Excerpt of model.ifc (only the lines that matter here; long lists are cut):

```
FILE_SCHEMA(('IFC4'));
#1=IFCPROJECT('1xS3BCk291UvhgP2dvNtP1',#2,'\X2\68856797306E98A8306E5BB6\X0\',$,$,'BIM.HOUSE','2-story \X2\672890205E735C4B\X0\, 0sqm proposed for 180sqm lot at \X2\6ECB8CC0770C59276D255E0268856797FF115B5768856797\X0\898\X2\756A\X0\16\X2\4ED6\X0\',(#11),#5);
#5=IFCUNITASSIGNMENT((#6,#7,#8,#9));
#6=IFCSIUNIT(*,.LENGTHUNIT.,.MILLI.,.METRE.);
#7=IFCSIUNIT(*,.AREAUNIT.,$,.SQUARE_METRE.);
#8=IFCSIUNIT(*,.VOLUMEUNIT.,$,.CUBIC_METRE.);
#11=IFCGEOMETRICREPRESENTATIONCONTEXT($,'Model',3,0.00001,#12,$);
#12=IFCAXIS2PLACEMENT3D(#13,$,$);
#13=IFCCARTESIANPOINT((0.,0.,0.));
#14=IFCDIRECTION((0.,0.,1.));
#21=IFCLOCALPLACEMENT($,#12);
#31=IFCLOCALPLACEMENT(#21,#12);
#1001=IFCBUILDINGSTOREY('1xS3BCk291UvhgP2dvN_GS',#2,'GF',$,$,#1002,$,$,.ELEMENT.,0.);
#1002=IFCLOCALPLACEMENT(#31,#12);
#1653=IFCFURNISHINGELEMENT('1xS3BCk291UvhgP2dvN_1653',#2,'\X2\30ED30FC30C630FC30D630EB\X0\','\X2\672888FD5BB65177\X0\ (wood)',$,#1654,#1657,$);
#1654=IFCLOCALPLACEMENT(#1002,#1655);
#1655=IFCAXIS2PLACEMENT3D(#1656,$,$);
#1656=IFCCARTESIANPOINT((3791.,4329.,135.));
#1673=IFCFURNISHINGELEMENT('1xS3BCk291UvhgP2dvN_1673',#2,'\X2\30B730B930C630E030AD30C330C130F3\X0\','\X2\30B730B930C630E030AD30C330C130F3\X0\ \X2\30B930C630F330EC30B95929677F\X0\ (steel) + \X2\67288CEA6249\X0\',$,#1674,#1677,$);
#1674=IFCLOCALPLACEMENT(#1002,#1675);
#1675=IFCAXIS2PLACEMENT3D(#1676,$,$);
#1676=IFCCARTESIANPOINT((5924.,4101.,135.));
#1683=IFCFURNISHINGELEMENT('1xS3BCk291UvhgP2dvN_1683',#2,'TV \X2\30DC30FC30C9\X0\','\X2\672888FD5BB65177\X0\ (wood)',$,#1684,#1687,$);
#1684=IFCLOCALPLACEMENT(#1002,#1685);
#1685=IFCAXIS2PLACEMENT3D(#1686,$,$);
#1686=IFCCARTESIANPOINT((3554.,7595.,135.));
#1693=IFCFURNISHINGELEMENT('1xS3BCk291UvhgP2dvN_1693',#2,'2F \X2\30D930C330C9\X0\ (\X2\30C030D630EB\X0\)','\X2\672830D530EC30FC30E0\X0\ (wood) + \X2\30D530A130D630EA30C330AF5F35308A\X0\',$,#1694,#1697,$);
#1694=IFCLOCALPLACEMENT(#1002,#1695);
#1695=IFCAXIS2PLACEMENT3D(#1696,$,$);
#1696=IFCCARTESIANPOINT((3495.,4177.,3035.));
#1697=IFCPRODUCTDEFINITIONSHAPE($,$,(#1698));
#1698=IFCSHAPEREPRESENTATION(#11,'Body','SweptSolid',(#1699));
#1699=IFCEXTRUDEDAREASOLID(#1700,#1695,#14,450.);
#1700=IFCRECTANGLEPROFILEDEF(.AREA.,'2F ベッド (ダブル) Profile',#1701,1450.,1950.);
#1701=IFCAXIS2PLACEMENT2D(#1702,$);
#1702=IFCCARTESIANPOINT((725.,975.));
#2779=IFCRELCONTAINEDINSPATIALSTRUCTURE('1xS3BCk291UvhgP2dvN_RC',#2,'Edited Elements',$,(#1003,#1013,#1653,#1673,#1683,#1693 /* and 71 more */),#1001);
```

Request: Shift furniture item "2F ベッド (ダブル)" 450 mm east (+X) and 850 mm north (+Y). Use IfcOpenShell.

```python
import ifcopenshell
import ifcopenshell.api.geometry
import ifcopenshell.util.placement
import ifcopenshell.util.unit

model = ifcopenshell.open("model.ifc")
unit_scale = ifcopenshell.util.unit.calculate_unit_scale(model)

item = model.by_id(1693)
matrix = ifcopenshell.util.placement.get_local_placement(item.ObjectPlacement)
matrix[0, 3] += 0.45 / unit_scale
matrix[1, 3] += 0.85 / unit_scale
ifcopenshell.api.geometry.edit_object_placement(model, product=item, matrix=matrix, is_si=False)

print(ifcopenshell.util.placement.get_local_placement(item.ObjectPlacement).round(3) + 0.0)

model.write("model_updated.ifc")
```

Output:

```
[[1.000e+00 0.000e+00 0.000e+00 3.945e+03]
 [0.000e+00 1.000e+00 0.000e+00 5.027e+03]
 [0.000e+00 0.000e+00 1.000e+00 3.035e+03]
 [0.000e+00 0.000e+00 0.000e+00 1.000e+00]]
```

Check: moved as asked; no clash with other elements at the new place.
